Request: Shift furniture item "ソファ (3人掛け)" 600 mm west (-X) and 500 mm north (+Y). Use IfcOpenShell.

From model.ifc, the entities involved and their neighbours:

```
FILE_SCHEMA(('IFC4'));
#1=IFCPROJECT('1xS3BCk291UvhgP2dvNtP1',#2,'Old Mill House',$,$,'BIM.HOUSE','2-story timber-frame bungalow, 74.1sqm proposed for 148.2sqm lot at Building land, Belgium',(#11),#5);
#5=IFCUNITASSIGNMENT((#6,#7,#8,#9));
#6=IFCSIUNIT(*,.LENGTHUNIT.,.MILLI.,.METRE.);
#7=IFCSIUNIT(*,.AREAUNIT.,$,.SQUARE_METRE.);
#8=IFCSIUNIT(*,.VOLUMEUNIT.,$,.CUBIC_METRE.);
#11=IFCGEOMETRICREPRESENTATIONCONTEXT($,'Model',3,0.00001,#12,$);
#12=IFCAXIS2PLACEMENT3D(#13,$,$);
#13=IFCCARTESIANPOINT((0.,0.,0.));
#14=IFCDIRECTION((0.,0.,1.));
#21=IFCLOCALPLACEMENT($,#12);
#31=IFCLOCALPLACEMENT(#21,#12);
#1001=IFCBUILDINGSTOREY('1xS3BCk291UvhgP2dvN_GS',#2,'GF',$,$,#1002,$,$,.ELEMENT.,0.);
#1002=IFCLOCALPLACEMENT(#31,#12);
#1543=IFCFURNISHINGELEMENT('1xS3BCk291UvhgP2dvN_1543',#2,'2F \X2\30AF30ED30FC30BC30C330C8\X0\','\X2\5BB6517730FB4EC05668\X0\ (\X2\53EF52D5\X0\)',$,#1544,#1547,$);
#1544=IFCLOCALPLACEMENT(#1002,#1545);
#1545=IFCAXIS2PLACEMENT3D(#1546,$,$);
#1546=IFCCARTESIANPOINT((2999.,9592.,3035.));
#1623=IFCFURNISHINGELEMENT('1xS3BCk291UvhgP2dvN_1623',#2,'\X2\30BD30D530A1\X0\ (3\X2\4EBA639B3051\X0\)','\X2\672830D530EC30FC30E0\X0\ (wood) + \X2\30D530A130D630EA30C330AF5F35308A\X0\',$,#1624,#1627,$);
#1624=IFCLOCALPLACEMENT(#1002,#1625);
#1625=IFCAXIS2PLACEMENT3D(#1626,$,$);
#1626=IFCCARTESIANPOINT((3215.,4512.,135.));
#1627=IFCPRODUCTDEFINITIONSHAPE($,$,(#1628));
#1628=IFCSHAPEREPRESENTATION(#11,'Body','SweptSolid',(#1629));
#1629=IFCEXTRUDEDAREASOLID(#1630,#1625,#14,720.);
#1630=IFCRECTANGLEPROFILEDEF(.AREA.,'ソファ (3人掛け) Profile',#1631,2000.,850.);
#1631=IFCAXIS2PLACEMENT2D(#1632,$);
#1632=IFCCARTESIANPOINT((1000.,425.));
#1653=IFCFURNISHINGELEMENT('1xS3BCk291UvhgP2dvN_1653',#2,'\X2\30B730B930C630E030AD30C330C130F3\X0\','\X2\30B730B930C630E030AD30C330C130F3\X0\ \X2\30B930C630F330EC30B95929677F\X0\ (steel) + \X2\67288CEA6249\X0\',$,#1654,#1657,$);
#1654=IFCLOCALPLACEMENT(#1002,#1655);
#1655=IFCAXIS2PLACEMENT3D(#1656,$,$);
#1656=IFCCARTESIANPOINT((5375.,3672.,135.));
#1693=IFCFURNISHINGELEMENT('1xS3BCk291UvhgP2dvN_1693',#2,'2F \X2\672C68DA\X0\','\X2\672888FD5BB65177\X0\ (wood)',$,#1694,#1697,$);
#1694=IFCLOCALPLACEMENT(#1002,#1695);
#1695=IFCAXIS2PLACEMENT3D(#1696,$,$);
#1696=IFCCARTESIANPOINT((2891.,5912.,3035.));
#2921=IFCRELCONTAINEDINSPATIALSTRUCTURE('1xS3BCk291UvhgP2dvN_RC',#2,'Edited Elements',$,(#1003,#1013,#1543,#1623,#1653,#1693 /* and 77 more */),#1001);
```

```python
import ifcopenshell
import ifcopenshell.api.geometry
import ifcopenshell.util.placement
import ifcopenshell.util.unit

model = ifcopenshell.open("model.ifc")
unit_scale = ifcopenshell.util.unit.calculate_unit_scale(model)

item = model.by_guid("1xS3BCk291UvhgP2dvN_1623")
matrix = ifcopenshell.util.placement.get_local_placement(item.ObjectPlacement)
matrix[0, 3] -= 0.6 / unit_scale
matrix[1, 3] += 0.5 / unit_scale
ifcopenshell.api.geometry.edit_object_placement(model, product=item, matrix=matrix, is_si=False)

print(ifcopenshell.util.placement.get_local_placement(item.ObjectPlacement).round(3) + 0.0)

model.write("model_rev.ifc")
```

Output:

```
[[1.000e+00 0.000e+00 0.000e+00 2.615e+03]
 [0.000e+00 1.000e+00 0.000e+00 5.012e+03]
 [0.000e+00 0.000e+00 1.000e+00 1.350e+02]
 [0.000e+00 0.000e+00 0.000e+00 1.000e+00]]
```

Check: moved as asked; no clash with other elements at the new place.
